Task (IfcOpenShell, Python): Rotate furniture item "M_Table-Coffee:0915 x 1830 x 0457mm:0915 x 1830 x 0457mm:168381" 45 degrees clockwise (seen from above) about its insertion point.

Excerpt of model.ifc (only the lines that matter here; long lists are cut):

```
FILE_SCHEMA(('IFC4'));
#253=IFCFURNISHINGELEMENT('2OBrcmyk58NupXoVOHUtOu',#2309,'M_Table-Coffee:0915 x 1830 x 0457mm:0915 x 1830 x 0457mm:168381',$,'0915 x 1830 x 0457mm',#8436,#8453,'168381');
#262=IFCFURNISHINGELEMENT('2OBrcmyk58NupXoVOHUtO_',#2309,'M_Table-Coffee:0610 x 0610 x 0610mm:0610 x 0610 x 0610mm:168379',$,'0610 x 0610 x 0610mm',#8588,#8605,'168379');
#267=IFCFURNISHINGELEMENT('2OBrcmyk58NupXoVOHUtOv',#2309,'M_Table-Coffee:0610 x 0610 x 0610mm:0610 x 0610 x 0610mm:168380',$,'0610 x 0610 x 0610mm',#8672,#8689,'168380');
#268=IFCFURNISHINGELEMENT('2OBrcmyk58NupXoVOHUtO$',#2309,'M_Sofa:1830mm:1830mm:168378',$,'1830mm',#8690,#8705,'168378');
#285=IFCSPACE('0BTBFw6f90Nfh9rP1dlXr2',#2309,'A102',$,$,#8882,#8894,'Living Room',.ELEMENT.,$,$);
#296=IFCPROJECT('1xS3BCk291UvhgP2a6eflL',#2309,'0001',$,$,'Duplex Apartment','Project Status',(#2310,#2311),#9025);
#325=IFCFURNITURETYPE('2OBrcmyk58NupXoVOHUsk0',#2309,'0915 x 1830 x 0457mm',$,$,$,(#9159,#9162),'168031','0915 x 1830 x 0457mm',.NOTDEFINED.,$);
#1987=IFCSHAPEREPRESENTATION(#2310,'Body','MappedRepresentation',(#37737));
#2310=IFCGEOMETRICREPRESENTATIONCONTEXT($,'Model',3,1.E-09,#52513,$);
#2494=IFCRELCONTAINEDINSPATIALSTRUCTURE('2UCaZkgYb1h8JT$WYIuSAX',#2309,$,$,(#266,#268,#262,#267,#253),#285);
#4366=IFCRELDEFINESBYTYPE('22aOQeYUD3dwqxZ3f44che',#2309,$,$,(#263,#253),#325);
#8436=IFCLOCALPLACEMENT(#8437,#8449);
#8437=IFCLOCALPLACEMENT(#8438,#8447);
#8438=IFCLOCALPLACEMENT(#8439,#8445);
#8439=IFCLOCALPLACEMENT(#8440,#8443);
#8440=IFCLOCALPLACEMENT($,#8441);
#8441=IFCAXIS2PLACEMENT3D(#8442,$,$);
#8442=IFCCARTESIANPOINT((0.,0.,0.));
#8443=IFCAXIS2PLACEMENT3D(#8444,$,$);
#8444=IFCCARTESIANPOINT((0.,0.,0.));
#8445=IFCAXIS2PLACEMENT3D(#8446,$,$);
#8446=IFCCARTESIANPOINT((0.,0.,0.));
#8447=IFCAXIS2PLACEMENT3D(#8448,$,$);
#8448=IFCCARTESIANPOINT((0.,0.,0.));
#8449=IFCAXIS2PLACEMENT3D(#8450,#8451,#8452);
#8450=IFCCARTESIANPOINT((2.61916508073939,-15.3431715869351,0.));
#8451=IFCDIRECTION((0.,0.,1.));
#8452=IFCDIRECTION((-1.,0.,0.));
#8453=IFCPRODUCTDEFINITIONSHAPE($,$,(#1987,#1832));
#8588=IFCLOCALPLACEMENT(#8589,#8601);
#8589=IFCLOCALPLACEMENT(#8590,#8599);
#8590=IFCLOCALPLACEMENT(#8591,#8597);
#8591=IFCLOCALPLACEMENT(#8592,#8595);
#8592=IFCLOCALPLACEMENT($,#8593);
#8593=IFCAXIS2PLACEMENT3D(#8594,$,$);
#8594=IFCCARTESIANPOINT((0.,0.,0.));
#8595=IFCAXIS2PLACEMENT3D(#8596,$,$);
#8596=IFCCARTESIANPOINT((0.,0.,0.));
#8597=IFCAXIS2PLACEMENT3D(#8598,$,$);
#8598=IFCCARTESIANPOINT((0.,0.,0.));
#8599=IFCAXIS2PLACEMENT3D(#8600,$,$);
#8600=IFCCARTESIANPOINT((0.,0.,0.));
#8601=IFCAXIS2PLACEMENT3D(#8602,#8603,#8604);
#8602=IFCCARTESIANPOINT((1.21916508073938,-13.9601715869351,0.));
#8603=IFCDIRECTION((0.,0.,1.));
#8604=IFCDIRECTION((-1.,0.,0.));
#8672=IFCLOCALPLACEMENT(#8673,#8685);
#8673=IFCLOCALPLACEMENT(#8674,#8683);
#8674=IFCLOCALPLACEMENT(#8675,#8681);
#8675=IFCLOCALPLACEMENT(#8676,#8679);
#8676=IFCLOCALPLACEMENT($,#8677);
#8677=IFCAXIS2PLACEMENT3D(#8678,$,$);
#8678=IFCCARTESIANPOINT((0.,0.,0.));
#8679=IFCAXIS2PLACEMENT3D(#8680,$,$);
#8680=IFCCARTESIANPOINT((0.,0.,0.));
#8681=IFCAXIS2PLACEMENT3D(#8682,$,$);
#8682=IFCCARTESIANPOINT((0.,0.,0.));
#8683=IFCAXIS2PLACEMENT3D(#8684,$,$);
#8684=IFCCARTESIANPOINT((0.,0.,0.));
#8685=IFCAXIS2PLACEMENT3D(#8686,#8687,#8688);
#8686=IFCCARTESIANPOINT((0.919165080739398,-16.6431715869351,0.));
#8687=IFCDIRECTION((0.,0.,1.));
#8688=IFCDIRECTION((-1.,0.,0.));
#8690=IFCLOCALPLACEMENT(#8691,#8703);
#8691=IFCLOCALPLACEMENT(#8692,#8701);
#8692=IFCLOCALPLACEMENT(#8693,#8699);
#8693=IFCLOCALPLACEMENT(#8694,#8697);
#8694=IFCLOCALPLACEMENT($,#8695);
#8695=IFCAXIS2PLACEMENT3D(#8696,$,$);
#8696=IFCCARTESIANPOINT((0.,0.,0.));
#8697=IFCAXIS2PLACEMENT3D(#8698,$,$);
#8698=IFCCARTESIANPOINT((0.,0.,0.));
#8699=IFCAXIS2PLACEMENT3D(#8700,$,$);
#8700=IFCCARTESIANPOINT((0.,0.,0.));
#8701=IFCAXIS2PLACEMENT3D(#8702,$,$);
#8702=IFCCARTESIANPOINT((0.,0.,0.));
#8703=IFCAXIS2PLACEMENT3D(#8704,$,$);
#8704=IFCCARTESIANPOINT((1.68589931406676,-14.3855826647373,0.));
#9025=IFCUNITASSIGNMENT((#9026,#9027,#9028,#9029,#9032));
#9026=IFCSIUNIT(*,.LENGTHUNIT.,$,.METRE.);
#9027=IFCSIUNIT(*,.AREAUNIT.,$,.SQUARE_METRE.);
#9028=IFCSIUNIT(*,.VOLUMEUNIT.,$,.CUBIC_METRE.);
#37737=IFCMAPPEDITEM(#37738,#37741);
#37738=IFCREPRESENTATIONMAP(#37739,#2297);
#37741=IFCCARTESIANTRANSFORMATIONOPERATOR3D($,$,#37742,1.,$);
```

```python
import ifcopenshell
import ifcopenshell.api.geometry
import ifcopenshell.util.placement

model = ifcopenshell.open("model.ifc")

item = model.by_guid("2OBrcmyk58NupXoVOHUtOu")
matrix = ifcopenshell.util.placement.get_local_placement(item.ObjectPlacement)
matrix = matrix @ ifcopenshell.util.placement.rotation(-45, "Z")
ifcopenshell.api.geometry.edit_object_placement(model, product=item, matrix=matrix, is_si=False)

print(ifcopenshell.util.placement.get_local_placement(item.ObjectPlacement).round(3) + 0.0)

model.write("model_edited.ifc")
```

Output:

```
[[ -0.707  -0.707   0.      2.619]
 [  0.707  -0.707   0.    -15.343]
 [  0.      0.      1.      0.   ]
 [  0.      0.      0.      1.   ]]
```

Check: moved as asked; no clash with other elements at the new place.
